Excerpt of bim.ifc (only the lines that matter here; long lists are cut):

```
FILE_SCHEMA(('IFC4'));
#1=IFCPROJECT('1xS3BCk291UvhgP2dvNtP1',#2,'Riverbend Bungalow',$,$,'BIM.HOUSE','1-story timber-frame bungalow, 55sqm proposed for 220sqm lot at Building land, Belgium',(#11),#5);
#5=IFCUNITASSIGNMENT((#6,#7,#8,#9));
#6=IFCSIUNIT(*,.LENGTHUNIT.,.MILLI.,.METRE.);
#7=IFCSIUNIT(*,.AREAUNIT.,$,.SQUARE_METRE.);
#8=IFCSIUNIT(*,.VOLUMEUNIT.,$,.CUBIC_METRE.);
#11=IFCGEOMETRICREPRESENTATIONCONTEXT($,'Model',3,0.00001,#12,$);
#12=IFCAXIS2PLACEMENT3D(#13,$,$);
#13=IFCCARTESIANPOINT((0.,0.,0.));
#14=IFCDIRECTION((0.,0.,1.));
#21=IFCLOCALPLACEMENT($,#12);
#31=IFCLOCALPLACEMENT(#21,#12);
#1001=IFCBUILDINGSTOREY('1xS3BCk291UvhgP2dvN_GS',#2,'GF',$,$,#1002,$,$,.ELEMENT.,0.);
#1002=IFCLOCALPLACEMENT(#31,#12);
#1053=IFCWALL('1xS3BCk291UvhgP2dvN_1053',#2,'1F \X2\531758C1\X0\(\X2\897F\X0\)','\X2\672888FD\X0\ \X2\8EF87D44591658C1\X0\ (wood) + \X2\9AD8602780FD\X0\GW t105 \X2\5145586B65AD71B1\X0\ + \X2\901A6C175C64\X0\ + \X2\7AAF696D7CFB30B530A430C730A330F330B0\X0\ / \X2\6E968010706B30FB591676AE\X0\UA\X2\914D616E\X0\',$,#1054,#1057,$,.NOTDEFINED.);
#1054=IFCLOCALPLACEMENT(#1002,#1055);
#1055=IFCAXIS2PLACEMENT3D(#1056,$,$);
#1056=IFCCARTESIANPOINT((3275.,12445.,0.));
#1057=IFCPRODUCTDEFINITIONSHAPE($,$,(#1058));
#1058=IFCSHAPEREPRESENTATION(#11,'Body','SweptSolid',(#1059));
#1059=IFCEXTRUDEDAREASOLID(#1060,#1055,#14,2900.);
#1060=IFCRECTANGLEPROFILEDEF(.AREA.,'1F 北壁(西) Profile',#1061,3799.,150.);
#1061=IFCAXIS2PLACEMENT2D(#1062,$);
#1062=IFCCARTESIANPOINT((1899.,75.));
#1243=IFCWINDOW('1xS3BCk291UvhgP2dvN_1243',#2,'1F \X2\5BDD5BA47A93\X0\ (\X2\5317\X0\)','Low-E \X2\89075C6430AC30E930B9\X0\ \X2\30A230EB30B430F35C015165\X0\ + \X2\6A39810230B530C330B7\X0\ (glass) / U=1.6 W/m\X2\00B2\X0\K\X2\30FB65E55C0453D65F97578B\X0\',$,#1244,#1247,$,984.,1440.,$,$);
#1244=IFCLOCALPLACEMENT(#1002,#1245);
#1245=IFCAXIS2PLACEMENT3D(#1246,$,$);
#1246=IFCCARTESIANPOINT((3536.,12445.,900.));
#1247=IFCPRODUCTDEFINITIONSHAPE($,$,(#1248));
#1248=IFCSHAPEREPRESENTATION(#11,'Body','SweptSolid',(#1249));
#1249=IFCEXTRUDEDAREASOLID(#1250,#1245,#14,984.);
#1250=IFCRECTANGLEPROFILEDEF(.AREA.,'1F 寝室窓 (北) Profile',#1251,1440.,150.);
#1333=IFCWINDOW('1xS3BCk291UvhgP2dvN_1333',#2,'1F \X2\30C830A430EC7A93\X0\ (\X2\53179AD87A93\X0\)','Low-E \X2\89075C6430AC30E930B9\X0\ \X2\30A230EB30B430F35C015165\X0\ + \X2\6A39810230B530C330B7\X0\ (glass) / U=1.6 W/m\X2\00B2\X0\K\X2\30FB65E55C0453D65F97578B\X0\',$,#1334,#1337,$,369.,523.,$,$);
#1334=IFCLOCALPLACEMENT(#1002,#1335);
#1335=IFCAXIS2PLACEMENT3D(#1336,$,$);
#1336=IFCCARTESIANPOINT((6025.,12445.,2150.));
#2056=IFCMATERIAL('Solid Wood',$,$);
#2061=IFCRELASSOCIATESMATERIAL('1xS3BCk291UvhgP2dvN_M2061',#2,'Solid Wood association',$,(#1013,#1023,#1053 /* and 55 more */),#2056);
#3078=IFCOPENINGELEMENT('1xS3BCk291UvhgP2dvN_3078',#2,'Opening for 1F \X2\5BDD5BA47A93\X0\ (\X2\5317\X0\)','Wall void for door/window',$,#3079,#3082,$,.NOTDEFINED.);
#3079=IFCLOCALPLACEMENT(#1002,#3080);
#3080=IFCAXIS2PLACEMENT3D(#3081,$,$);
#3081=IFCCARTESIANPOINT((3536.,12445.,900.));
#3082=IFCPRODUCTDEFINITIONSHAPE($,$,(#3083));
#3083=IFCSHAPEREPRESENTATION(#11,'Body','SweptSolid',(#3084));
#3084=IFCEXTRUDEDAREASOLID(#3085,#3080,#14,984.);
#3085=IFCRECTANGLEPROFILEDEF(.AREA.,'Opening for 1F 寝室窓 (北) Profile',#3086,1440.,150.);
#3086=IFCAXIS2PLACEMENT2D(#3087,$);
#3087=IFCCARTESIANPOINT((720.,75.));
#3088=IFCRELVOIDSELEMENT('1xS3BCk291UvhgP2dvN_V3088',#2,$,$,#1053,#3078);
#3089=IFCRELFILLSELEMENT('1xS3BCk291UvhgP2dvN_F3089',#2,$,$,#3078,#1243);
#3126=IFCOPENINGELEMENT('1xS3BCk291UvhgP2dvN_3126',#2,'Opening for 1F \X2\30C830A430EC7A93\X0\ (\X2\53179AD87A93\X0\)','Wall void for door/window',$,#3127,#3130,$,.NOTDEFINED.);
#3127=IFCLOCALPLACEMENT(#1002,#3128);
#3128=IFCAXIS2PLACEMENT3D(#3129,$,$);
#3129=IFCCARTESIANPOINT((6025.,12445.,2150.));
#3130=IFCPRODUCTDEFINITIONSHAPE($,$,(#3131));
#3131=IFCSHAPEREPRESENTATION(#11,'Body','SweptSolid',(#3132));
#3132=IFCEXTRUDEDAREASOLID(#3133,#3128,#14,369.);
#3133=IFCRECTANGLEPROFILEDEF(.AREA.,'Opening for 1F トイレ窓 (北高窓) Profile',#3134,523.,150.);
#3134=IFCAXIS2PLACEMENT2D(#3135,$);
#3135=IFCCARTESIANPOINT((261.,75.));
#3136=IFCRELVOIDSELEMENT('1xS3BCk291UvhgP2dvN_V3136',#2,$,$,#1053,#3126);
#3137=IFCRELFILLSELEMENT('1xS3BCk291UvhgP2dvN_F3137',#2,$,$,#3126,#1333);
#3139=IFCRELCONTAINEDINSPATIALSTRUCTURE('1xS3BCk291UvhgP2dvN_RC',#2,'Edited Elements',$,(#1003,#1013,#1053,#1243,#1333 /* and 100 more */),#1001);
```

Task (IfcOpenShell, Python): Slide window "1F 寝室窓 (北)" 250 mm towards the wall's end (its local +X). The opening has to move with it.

```python
import ifcopenshell
import ifcopenshell.api.geometry
import ifcopenshell.util.placement

model = ifcopenshell.open("bim.ifc")

window = model.by_guid("1xS3BCk291UvhgP2dvN_1243")
opening = window.FillsVoids[0].RelatingOpeningElement
wall = opening.VoidsElements[0].RelatingBuildingElement

wall_matrix = ifcopenshell.util.placement.get_local_placement(wall.ObjectPlacement)
shift = wall_matrix[:3, 0] * 250.0
before = ifcopenshell.util.placement.get_local_placement(window.ObjectPlacement)[:3, 3].copy()

# The window is not placed relative to its opening, so move both.
for product in (opening, window):
    matrix = ifcopenshell.util.placement.get_local_placement(product.ObjectPlacement)
    matrix[:3, 3] += shift
    ifcopenshell.api.geometry.edit_object_placement(model, product=product, matrix=matrix, is_si=False)

after = ifcopenshell.util.placement.get_local_placement(window.ObjectPlacement)[:3, 3]
print("window moved by", (after - before).round(3) + 0.0)

model.write("bim-out.ifc")
```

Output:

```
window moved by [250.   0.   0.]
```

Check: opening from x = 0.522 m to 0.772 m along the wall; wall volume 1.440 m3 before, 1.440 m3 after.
